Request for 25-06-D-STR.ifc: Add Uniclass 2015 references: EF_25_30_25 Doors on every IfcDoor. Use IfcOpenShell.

First a look at what the model holds.

```python
import ifcopenshell

model = ifcopenshell.open("25-06-D-STR.ifc")
print(model.schema)
print("classifications:", [c.Name for c in model.by_type("IfcClassification")])
for ifc_class in ("IfcDoor", "IfcRoof", "IfcStair", "IfcWall", "IfcWindow"):
    print(ifc_class, len(model.by_type(ifc_class)))
```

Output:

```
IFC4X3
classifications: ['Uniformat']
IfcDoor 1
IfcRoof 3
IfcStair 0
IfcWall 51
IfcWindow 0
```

```python
import ifcopenshell
import ifcopenshell.api.classification

model = ifcopenshell.open("25-06-D-STR.ifc")

system = ifcopenshell.api.classification.add_classification(model, classification="Uniclass 2015")

codes = {
    "IfcDoor": ("EF_25_30_25", "Doors"),
}
for ifc_class, (code, name) in codes.items():
    products = model.by_type(ifc_class)
    ifcopenshell.api.classification.add_reference(
        model, products=products, classification=system, identification=code, name=name
    )
    print(code, len(products))

model.write("25-06-D-STR_edited.ifc")
```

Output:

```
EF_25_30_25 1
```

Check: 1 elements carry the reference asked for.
